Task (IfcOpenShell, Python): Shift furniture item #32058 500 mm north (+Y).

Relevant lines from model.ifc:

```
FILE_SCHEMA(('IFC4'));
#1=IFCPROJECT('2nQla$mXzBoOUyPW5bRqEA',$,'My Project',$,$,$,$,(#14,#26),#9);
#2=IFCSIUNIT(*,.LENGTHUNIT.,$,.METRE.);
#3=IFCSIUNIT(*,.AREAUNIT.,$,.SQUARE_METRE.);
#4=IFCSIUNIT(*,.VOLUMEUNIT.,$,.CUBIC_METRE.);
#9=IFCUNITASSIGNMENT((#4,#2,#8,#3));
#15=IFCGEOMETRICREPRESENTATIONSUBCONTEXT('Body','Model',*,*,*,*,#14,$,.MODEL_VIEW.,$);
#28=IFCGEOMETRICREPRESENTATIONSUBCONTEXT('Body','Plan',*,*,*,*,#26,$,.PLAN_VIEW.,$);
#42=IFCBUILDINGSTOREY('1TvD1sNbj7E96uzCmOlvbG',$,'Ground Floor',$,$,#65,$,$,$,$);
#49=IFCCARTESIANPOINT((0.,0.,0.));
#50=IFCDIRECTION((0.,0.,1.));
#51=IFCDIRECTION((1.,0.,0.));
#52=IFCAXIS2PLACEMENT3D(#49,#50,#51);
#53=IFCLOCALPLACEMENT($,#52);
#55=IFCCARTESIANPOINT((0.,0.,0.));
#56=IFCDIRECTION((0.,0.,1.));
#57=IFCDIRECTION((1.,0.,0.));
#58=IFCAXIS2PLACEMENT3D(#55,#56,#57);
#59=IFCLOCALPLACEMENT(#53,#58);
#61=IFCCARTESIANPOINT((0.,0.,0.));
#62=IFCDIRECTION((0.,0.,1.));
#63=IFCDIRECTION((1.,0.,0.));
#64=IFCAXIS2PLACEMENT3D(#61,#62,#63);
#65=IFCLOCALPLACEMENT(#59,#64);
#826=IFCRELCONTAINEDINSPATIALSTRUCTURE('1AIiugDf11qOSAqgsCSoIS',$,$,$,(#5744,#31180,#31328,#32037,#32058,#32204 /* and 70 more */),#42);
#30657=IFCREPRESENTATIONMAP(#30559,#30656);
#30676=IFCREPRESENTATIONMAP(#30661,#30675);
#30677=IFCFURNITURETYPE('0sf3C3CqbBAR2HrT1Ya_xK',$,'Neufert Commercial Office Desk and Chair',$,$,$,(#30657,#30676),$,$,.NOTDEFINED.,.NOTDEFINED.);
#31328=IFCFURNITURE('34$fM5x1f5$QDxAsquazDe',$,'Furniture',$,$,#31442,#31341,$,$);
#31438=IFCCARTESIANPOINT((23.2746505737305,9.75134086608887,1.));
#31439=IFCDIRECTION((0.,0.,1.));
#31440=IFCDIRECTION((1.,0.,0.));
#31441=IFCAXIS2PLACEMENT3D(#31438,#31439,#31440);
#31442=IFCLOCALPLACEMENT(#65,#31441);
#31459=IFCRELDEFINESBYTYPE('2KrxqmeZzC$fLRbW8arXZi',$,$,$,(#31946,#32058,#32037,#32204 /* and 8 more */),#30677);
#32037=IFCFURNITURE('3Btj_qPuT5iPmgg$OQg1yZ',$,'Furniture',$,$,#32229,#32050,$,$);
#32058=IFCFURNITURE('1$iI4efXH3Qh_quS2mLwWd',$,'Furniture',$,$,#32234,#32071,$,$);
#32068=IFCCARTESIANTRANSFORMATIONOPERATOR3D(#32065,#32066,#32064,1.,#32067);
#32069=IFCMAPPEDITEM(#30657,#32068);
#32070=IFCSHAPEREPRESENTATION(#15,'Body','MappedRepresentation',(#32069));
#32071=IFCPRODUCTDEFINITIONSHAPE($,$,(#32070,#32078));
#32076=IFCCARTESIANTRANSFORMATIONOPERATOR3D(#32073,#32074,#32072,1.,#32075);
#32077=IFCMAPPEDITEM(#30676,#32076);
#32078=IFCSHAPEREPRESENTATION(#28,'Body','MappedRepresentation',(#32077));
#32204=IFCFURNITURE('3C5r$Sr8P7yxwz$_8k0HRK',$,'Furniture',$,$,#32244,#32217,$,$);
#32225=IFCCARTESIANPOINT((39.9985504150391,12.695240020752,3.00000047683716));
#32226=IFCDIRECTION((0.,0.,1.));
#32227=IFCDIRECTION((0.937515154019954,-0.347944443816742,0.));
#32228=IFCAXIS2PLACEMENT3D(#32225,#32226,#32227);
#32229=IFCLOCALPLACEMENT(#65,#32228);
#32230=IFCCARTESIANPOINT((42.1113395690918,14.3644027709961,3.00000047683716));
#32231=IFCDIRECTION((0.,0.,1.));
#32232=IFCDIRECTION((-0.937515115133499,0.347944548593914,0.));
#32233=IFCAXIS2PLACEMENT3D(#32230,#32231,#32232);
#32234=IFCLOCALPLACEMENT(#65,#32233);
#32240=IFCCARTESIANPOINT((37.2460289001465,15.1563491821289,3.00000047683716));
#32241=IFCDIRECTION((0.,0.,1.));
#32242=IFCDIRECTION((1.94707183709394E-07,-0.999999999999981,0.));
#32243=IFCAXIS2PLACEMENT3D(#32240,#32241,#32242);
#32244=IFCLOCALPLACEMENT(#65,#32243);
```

```python
import ifcopenshell
import ifcopenshell.api.geometry
import ifcopenshell.util.placement
import ifcopenshell.util.unit

model = ifcopenshell.open("model.ifc")
unit_scale = ifcopenshell.util.unit.calculate_unit_scale(model)

item = model.by_guid("1$iI4efXH3Qh_quS2mLwWd")
matrix = ifcopenshell.util.placement.get_local_placement(item.ObjectPlacement)
matrix[1, 3] += 0.5 / unit_scale
ifcopenshell.api.geometry.edit_object_placement(model, product=item, matrix=matrix, is_si=False)

print(ifcopenshell.util.placement.get_local_placement(item.ObjectPlacement).round(3) + 0.0)

model.write("model-out.ifc")
```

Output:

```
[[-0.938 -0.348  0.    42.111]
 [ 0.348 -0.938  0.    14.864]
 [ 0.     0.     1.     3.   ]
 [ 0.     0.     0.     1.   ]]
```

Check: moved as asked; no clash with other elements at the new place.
